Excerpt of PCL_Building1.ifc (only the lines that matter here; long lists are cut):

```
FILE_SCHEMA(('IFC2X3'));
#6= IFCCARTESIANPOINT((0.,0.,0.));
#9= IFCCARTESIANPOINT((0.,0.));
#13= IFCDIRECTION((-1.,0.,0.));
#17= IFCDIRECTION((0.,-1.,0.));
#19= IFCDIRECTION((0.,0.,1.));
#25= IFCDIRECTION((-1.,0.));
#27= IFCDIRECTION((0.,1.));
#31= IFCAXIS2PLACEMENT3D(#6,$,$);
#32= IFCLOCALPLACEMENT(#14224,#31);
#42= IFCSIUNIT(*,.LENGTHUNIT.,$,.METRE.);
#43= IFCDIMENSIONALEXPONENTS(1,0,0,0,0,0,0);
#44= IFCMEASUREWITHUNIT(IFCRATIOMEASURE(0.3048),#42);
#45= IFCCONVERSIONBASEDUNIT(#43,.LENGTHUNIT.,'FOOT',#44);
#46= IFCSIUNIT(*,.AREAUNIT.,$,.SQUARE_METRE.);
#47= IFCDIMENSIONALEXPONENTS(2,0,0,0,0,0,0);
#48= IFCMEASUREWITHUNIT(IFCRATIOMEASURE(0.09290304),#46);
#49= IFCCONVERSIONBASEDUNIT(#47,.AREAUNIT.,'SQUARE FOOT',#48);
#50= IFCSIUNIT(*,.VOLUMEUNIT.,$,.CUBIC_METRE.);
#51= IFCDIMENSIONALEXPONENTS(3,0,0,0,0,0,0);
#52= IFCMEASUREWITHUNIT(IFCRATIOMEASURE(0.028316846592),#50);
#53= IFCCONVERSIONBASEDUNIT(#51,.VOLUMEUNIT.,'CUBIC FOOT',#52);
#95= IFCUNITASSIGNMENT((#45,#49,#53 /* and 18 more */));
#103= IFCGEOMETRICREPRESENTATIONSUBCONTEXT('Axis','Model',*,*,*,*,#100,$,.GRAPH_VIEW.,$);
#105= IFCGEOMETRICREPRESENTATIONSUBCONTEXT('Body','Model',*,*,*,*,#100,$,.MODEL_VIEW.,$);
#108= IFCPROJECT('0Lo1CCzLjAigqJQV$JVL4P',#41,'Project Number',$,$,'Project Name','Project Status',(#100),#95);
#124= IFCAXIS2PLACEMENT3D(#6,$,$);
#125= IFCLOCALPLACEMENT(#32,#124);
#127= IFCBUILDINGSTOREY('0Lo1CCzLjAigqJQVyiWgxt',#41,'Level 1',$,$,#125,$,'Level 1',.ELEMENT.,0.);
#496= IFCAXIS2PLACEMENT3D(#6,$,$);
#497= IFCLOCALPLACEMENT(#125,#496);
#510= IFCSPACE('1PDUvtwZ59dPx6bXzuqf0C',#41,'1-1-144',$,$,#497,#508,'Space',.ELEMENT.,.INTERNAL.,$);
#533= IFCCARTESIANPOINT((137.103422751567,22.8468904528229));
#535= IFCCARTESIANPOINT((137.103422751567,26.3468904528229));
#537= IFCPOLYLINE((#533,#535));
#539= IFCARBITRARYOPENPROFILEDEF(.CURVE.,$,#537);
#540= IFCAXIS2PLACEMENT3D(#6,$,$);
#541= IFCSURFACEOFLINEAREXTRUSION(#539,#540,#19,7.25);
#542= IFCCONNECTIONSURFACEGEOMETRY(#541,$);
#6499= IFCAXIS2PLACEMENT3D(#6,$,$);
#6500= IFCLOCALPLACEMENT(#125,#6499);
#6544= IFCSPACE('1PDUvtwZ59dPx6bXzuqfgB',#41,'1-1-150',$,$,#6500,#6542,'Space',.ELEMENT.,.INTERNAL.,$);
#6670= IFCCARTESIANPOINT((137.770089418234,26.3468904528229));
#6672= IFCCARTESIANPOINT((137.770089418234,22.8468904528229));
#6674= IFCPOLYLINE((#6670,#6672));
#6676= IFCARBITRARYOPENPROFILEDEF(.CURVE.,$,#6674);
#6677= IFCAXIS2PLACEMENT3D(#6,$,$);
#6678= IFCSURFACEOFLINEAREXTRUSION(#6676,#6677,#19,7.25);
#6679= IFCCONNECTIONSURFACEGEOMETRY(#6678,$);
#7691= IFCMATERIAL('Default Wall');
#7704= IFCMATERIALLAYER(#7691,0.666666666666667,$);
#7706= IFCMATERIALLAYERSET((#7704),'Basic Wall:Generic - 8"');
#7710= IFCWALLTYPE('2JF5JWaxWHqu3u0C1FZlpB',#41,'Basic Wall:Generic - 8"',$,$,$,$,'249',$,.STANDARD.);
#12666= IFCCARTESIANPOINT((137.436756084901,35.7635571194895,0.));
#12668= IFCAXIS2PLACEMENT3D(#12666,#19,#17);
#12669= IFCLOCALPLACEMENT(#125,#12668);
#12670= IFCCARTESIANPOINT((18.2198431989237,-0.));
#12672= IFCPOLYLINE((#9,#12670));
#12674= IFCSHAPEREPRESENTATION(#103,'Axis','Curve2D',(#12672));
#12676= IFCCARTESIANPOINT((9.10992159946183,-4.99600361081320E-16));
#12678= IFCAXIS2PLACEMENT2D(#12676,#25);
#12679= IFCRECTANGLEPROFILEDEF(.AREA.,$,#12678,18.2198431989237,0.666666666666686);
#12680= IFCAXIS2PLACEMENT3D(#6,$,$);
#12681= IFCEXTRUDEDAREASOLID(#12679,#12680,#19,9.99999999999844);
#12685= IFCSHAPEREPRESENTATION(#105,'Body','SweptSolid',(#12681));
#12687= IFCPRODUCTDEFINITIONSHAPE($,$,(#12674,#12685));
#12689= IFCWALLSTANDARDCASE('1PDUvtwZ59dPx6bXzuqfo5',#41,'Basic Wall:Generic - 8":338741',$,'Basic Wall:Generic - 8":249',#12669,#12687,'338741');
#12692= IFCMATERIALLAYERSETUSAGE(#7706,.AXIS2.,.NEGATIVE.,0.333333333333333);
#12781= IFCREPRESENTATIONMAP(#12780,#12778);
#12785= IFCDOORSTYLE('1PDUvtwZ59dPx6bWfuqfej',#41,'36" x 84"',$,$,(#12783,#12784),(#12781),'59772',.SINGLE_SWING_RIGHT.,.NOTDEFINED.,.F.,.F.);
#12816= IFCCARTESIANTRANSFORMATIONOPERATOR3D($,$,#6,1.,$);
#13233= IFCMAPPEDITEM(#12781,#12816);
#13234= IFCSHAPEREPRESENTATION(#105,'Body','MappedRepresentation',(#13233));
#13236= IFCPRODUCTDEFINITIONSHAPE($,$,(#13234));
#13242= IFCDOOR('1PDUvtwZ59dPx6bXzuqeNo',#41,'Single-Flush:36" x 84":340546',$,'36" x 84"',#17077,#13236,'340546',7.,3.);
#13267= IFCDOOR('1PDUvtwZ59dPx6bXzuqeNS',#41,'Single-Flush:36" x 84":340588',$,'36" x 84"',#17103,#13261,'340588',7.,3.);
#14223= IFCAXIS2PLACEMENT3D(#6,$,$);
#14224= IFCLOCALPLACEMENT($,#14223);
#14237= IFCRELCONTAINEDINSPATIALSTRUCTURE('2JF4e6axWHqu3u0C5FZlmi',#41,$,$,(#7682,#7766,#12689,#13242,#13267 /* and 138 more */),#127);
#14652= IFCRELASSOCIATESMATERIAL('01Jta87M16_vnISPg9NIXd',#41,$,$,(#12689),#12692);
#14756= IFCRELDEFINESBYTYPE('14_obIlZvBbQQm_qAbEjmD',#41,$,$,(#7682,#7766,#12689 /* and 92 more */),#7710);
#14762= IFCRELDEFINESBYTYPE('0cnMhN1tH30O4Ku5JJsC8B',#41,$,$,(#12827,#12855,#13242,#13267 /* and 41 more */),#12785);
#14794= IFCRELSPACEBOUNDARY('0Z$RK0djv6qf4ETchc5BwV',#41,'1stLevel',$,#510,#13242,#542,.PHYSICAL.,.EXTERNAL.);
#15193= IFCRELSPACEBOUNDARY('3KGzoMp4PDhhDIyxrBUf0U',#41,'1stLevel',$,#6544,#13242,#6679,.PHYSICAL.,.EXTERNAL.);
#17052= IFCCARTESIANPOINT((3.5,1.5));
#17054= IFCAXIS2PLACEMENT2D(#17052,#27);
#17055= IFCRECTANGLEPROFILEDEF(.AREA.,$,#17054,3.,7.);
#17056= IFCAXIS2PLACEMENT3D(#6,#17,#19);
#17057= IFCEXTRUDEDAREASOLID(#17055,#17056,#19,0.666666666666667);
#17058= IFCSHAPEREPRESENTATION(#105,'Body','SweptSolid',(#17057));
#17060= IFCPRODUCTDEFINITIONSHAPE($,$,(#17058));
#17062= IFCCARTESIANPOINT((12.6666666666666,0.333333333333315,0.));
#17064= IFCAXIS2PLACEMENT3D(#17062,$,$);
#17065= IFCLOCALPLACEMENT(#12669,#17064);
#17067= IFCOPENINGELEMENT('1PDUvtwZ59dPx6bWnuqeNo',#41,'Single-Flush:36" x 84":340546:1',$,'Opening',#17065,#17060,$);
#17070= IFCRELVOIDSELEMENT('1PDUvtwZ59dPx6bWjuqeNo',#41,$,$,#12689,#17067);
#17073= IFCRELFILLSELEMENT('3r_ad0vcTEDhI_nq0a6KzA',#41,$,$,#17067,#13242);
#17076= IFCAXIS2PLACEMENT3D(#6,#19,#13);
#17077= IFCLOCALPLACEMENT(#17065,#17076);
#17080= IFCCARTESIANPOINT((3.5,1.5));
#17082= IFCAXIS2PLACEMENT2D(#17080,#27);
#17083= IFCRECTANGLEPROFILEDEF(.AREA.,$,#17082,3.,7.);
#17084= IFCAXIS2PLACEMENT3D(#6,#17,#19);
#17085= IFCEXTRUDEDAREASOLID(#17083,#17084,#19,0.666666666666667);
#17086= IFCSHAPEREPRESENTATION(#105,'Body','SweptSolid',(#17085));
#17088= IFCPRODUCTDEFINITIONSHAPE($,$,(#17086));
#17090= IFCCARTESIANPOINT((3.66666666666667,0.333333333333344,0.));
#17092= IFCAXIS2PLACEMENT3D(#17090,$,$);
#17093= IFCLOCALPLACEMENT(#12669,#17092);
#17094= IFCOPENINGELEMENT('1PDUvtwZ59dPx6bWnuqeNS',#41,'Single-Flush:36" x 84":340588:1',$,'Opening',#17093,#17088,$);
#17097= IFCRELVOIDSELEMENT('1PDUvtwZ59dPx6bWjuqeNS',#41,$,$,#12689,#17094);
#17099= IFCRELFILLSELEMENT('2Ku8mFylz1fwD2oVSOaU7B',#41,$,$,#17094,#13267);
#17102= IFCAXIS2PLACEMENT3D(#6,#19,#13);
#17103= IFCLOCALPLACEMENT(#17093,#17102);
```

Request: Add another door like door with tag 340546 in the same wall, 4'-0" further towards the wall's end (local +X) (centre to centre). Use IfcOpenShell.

```python
import numpy as np
import ifcopenshell
import ifcopenshell.api.feature
import ifcopenshell.api.geometry
import ifcopenshell.api.root
import ifcopenshell.geom
import ifcopenshell.util.element
import ifcopenshell.util.placement
import ifcopenshell.util.shape
import ifcopenshell.util.unit

model = ifcopenshell.open("PCL_Building1.ifc")
unit_scale = ifcopenshell.util.unit.calculate_unit_scale(model)
settings = ifcopenshell.geom.settings()


def volume(element):
    """Net volume in cubic metres, openings subtracted."""
    shape = ifcopenshell.geom.create_shape(settings, element)
    return ifcopenshell.util.shape.get_volume(shape.geometry)


def reuse_history(source, copy):
    """copy_class also copies each property set's owner history, people and application; keep the originals."""
    for rel in copy.IsDefinedBy:
        if rel.is_a("IfcRelDefinesByProperties") and (history := rel.RelatingPropertyDefinition.OwnerHistory):
            rel.RelatingPropertyDefinition.OwnerHistory = source.OwnerHistory
            ifcopenshell.util.element.remove_deep2(model, history)


door = model.by_id(13242)
opening = door.FillsVoids[0].RelatingOpeningElement
wall = opening.VoidsElements[0].RelatingBuildingElement
before = volume(wall)
shift = ifcopenshell.util.placement.get_local_placement(wall.ObjectPlacement)[:3, 0] * 48 * 0.0254 / unit_scale

# copy_class copies the void relationship, type, container and properties, but no geometry.
new_opening = ifcopenshell.api.root.copy_class(model, product=opening)
new_opening.Representation = ifcopenshell.util.element.copy_deep(
    model, opening.Representation, exclude=["IfcGeometricRepresentationContext", "IfcRepresentationMap"]
)
new_opening.Name = 'Single-Flush:36" x 84"'
new_door = ifcopenshell.api.root.copy_class(model, product=door)
new_door.Representation = ifcopenshell.util.element.copy_deep(
    model, door.Representation, exclude=["IfcGeometricRepresentationContext", "IfcRepresentationMap"]
)
new_door.Name = 'Single-Flush:36" x 84"'
new_door.Tag = None
reuse_history(door, new_door)
fills = ifcopenshell.api.feature.add_filling(model, opening=new_opening, element=new_door)
fills.OwnerHistory = new_door.OwnerHistory  # required in IFC2X3

for old, new in ((opening, new_opening), (door, new_door)):
    matrix = ifcopenshell.util.placement.get_local_placement(old.ObjectPlacement)
    matrix[:3, 3] += shift
    ifcopenshell.api.geometry.edit_object_placement(model, product=new, matrix=matrix, is_si=False)

# The copied space boundaries still share their surfaces with the original.
for rel in new_door.ProvidesBoundaries:
    if rel.ConnectionGeometry:
        rel.ConnectionGeometry = ifcopenshell.util.element.copy_deep(model, rel.ConnectionGeometry)

# Space boundary surfaces are stored in each space's coordinates; move them too.
for rel in new_door.ProvidesBoundaries:
    if not rel.ConnectionGeometry:
        continue
    surface = rel.ConnectionGeometry.SurfaceOnRelatingElement
    space_matrix = ifcopenshell.util.placement.get_local_placement(rel.RelatingSpace.ObjectPlacement)
    point = np.array(surface.Position.Location.Coordinates) + space_matrix[:3, :3].T @ shift
    surface.Position = model.createIfcAxis2Placement3D(
        model.createIfcCartesianPoint(point.tolist()), surface.Position.Axis, surface.Position.RefDirection
    )

after = volume(wall)

print(f"wall volume {before:.3f} -> {after:.3f} m3")

model.write("PCL_Building1-out.ifc")
```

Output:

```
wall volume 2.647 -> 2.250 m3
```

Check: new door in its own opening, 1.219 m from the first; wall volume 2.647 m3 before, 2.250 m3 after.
